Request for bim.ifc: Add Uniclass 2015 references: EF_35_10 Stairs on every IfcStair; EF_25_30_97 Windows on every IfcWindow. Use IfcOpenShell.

First a look at what the model holds.

```python
import ifcopenshell

model = ifcopenshell.open("bim.ifc")
print(model.schema)
print("classifications:", [c.Name for c in model.by_type("IfcClassification")])
for ifc_class in ("IfcDoor", "IfcRoof", "IfcStair", "IfcWall", "IfcWindow"):
    print(ifc_class, len(model.by_type(ifc_class)))
```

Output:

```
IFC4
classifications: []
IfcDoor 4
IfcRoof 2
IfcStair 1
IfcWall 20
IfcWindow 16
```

```python
import ifcopenshell
import ifcopenshell.api.classification

model = ifcopenshell.open("bim.ifc")

system = ifcopenshell.api.classification.add_classification(model, classification="Uniclass 2015")

codes = {
    "IfcStair": ("EF_35_10", "Stairs"),
    "IfcWindow": ("EF_25_30_97", "Windows"),
}
for ifc_class, (code, name) in codes.items():
    products = model.by_type(ifc_class)
    ifcopenshell.api.classification.add_reference(
        model, products=products, classification=system, identification=code, name=name
    )
    print(code, len(products))

model.write("bim_v2.ifc")
```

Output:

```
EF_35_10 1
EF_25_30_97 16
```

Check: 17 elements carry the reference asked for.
